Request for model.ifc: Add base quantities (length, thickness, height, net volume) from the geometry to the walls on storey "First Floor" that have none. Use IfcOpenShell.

First a look at what the model holds.

```python
import ifcopenshell
import ifcopenshell.util.element
import ifcopenshell.util.unit

model = ifcopenshell.open("model.ifc")
print(model.schema)
for unit_type in ("LENGTHUNIT", "AREAUNIT", "VOLUMEUNIT"):
    print(unit_type, ifcopenshell.util.unit.calculate_unit_scale(model, unit_type))
storey = next(s for s in model.by_type("IfcBuildingStorey") if s.Name == "First Floor")
walls = [e for e in ifcopenshell.util.element.get_decomposition(storey) if e.is_a("IfcWall")]
for e in sorted(walls, key=lambda e: e.id()):
    print(e.id(), e.is_a(), e.Name, list(ifcopenshell.util.element.get_psets(e, qtos_only=True)), sep=" | ")
```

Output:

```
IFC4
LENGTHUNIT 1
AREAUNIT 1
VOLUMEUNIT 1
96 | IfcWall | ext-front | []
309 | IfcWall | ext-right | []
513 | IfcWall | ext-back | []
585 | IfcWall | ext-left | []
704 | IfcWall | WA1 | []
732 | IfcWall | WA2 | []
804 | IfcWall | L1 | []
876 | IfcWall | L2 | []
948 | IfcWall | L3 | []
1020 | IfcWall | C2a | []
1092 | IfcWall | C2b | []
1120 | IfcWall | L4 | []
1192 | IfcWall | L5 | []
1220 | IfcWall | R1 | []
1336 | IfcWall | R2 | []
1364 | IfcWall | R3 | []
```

```python
import ifcopenshell
import ifcopenshell.api.pset
import ifcopenshell.geom
import ifcopenshell.util.element
import ifcopenshell.util.shape
import ifcopenshell.util.unit

model = ifcopenshell.open("model.ifc")
unit_scale = ifcopenshell.util.unit.calculate_unit_scale(model)
volume_scale = ifcopenshell.util.unit.calculate_unit_scale(model, "VOLUMEUNIT")
settings = ifcopenshell.geom.settings()

storey = next(s for s in model.by_type("IfcBuildingStorey") if s.Name == "First Floor")
walls = [e for e in ifcopenshell.util.element.get_decomposition(storey) if e.is_a("IfcWall")]

for e in sorted(walls, key=lambda e: e.id()):
    if ifcopenshell.util.element.get_psets(e, qtos_only=True, should_inherit=False):
        continue
    # Geometry comes back in metres, in the element's own axes.
    shape = ifcopenshell.geom.create_shape(settings, e)
    values = {
        "Length": ifcopenshell.util.shape.get_x(shape.geometry) / unit_scale,
        "Width": ifcopenshell.util.shape.get_y(shape.geometry) / unit_scale,
        "Height": ifcopenshell.util.shape.get_z(shape.geometry) / unit_scale,
        "NetVolume": ifcopenshell.util.shape.get_volume(shape.geometry) / volume_scale,
    }
    qto = ifcopenshell.api.pset.add_qto(model, product=e, name="Qto_WallBaseQuantities")
    ifcopenshell.api.pset.edit_qto(model, qto=qto, properties=values)
    print(e.id(), {k: round(v, 3) for k, v in values.items()})

model.write("model-out.ifc")
```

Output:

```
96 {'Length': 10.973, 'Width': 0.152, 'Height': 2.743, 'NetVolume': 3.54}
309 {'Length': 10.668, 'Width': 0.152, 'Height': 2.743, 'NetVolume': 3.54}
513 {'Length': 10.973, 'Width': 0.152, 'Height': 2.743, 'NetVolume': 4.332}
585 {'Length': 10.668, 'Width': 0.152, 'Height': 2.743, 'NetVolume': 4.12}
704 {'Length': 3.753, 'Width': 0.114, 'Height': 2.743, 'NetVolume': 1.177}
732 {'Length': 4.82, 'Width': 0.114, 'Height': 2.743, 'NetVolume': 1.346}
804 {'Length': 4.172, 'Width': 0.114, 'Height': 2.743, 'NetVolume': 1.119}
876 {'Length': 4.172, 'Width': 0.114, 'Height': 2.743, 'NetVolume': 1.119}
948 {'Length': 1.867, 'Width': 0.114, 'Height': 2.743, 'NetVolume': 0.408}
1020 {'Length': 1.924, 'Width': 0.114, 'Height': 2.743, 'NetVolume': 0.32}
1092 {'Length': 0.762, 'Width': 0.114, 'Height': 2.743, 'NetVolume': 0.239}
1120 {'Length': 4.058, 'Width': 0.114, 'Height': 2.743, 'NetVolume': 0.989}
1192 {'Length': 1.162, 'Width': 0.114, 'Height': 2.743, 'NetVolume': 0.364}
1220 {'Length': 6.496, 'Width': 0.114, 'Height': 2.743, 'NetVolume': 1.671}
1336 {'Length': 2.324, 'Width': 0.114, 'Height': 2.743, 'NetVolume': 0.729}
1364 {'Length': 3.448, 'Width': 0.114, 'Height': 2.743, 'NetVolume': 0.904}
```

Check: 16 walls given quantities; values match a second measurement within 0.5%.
